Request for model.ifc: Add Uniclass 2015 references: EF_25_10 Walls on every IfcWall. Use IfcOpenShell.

First a look at what the model holds.

```python
import ifcopenshell

model = ifcopenshell.open("model.ifc")
print(model.schema)
print("classifications:", [c.Name for c in model.by_type("IfcClassification")])
for ifc_class in ("IfcDoor", "IfcRoof", "IfcStair", "IfcWall", "IfcWindow"):
    print(ifc_class, len(model.by_type(ifc_class)))
```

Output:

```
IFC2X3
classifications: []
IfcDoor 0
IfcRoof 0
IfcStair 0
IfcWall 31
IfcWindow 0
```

```python
import ifcopenshell
import ifcopenshell.api.classification

model = ifcopenshell.open("model.ifc")

# IFC2X3 requires Source and Edition and has no link from the project to the system.
system = model.create_entity("IfcClassification", Source="NBS", Edition="2015", Name="Uniclass 2015")

codes = {
    "IfcWall": ("EF_25_10", "Walls"),
}
for ifc_class, (code, name) in codes.items():
    products = model.by_type(ifc_class)
    ifcopenshell.api.classification.add_reference(
        model, products=products, classification=system, identification=code, name=name
    )
    print(code, len(products))

model.write("model_rev.ifc")
```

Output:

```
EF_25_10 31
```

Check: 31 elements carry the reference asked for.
